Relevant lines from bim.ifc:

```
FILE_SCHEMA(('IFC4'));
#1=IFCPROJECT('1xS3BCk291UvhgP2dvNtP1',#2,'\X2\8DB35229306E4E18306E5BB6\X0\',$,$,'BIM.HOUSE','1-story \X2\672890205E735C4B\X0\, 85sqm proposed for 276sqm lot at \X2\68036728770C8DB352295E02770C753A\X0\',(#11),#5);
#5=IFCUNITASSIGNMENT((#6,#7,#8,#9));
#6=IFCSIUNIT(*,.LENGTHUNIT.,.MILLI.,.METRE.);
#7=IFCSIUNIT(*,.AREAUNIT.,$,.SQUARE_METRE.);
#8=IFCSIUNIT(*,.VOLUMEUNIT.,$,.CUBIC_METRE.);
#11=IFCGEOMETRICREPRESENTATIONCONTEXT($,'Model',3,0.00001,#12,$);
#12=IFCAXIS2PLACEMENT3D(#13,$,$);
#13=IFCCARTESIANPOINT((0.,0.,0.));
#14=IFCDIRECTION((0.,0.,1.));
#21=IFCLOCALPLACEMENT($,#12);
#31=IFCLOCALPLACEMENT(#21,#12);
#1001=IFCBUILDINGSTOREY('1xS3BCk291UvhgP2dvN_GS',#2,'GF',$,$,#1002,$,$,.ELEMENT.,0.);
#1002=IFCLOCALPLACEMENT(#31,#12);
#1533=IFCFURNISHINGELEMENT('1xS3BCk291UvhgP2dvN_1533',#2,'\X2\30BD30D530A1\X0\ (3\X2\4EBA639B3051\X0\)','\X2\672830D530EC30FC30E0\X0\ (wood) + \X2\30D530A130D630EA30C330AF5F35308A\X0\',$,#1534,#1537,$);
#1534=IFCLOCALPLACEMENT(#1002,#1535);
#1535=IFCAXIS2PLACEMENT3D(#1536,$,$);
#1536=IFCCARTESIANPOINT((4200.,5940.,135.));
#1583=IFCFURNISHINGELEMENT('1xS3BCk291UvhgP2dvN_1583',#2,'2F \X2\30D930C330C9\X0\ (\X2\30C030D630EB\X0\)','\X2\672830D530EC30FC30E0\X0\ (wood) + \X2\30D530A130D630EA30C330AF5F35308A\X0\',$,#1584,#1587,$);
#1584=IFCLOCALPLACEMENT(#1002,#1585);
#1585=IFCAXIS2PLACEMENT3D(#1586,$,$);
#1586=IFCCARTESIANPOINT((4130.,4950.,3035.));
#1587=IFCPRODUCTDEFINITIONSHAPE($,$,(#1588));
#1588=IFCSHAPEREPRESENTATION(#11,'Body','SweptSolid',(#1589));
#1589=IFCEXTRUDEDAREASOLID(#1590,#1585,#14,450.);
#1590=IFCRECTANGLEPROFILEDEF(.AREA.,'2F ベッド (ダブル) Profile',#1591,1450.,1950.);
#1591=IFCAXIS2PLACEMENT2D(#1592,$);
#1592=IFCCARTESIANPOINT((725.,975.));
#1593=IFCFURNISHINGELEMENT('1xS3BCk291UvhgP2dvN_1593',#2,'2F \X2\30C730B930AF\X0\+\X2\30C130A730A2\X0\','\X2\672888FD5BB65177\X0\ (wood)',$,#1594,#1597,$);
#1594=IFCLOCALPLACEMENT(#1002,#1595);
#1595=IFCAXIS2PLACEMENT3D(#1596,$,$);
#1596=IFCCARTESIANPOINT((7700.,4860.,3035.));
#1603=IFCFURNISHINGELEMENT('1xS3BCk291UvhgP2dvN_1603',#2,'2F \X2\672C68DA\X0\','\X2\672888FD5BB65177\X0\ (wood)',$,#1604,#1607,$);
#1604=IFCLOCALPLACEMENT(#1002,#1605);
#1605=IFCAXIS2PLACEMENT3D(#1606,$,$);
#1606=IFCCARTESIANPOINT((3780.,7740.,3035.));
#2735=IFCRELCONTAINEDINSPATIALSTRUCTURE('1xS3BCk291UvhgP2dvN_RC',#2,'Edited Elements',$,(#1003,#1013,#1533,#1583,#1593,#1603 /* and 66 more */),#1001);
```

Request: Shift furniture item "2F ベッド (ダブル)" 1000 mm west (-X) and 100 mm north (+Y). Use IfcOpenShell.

```python
import ifcopenshell
import ifcopenshell.api.geometry
import ifcopenshell.util.placement
import ifcopenshell.util.unit

model = ifcopenshell.open("bim.ifc")
unit_scale = ifcopenshell.util.unit.calculate_unit_scale(model)

item = model.by_guid("1xS3BCk291UvhgP2dvN_1583")
matrix = ifcopenshell.util.placement.get_local_placement(item.ObjectPlacement)
matrix[0, 3] -= 1 / unit_scale
matrix[1, 3] += 0.1 / unit_scale
ifcopenshell.api.geometry.edit_object_placement(model, product=item, matrix=matrix, is_si=False)

print(ifcopenshell.util.placement.get_local_placement(item.ObjectPlacement).round(3) + 0.0)

model.write("bim-out.ifc")
```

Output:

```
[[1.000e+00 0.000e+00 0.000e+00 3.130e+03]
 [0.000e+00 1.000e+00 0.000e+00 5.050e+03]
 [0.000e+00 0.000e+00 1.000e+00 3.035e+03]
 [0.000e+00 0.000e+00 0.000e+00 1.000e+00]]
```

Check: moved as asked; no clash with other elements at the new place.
